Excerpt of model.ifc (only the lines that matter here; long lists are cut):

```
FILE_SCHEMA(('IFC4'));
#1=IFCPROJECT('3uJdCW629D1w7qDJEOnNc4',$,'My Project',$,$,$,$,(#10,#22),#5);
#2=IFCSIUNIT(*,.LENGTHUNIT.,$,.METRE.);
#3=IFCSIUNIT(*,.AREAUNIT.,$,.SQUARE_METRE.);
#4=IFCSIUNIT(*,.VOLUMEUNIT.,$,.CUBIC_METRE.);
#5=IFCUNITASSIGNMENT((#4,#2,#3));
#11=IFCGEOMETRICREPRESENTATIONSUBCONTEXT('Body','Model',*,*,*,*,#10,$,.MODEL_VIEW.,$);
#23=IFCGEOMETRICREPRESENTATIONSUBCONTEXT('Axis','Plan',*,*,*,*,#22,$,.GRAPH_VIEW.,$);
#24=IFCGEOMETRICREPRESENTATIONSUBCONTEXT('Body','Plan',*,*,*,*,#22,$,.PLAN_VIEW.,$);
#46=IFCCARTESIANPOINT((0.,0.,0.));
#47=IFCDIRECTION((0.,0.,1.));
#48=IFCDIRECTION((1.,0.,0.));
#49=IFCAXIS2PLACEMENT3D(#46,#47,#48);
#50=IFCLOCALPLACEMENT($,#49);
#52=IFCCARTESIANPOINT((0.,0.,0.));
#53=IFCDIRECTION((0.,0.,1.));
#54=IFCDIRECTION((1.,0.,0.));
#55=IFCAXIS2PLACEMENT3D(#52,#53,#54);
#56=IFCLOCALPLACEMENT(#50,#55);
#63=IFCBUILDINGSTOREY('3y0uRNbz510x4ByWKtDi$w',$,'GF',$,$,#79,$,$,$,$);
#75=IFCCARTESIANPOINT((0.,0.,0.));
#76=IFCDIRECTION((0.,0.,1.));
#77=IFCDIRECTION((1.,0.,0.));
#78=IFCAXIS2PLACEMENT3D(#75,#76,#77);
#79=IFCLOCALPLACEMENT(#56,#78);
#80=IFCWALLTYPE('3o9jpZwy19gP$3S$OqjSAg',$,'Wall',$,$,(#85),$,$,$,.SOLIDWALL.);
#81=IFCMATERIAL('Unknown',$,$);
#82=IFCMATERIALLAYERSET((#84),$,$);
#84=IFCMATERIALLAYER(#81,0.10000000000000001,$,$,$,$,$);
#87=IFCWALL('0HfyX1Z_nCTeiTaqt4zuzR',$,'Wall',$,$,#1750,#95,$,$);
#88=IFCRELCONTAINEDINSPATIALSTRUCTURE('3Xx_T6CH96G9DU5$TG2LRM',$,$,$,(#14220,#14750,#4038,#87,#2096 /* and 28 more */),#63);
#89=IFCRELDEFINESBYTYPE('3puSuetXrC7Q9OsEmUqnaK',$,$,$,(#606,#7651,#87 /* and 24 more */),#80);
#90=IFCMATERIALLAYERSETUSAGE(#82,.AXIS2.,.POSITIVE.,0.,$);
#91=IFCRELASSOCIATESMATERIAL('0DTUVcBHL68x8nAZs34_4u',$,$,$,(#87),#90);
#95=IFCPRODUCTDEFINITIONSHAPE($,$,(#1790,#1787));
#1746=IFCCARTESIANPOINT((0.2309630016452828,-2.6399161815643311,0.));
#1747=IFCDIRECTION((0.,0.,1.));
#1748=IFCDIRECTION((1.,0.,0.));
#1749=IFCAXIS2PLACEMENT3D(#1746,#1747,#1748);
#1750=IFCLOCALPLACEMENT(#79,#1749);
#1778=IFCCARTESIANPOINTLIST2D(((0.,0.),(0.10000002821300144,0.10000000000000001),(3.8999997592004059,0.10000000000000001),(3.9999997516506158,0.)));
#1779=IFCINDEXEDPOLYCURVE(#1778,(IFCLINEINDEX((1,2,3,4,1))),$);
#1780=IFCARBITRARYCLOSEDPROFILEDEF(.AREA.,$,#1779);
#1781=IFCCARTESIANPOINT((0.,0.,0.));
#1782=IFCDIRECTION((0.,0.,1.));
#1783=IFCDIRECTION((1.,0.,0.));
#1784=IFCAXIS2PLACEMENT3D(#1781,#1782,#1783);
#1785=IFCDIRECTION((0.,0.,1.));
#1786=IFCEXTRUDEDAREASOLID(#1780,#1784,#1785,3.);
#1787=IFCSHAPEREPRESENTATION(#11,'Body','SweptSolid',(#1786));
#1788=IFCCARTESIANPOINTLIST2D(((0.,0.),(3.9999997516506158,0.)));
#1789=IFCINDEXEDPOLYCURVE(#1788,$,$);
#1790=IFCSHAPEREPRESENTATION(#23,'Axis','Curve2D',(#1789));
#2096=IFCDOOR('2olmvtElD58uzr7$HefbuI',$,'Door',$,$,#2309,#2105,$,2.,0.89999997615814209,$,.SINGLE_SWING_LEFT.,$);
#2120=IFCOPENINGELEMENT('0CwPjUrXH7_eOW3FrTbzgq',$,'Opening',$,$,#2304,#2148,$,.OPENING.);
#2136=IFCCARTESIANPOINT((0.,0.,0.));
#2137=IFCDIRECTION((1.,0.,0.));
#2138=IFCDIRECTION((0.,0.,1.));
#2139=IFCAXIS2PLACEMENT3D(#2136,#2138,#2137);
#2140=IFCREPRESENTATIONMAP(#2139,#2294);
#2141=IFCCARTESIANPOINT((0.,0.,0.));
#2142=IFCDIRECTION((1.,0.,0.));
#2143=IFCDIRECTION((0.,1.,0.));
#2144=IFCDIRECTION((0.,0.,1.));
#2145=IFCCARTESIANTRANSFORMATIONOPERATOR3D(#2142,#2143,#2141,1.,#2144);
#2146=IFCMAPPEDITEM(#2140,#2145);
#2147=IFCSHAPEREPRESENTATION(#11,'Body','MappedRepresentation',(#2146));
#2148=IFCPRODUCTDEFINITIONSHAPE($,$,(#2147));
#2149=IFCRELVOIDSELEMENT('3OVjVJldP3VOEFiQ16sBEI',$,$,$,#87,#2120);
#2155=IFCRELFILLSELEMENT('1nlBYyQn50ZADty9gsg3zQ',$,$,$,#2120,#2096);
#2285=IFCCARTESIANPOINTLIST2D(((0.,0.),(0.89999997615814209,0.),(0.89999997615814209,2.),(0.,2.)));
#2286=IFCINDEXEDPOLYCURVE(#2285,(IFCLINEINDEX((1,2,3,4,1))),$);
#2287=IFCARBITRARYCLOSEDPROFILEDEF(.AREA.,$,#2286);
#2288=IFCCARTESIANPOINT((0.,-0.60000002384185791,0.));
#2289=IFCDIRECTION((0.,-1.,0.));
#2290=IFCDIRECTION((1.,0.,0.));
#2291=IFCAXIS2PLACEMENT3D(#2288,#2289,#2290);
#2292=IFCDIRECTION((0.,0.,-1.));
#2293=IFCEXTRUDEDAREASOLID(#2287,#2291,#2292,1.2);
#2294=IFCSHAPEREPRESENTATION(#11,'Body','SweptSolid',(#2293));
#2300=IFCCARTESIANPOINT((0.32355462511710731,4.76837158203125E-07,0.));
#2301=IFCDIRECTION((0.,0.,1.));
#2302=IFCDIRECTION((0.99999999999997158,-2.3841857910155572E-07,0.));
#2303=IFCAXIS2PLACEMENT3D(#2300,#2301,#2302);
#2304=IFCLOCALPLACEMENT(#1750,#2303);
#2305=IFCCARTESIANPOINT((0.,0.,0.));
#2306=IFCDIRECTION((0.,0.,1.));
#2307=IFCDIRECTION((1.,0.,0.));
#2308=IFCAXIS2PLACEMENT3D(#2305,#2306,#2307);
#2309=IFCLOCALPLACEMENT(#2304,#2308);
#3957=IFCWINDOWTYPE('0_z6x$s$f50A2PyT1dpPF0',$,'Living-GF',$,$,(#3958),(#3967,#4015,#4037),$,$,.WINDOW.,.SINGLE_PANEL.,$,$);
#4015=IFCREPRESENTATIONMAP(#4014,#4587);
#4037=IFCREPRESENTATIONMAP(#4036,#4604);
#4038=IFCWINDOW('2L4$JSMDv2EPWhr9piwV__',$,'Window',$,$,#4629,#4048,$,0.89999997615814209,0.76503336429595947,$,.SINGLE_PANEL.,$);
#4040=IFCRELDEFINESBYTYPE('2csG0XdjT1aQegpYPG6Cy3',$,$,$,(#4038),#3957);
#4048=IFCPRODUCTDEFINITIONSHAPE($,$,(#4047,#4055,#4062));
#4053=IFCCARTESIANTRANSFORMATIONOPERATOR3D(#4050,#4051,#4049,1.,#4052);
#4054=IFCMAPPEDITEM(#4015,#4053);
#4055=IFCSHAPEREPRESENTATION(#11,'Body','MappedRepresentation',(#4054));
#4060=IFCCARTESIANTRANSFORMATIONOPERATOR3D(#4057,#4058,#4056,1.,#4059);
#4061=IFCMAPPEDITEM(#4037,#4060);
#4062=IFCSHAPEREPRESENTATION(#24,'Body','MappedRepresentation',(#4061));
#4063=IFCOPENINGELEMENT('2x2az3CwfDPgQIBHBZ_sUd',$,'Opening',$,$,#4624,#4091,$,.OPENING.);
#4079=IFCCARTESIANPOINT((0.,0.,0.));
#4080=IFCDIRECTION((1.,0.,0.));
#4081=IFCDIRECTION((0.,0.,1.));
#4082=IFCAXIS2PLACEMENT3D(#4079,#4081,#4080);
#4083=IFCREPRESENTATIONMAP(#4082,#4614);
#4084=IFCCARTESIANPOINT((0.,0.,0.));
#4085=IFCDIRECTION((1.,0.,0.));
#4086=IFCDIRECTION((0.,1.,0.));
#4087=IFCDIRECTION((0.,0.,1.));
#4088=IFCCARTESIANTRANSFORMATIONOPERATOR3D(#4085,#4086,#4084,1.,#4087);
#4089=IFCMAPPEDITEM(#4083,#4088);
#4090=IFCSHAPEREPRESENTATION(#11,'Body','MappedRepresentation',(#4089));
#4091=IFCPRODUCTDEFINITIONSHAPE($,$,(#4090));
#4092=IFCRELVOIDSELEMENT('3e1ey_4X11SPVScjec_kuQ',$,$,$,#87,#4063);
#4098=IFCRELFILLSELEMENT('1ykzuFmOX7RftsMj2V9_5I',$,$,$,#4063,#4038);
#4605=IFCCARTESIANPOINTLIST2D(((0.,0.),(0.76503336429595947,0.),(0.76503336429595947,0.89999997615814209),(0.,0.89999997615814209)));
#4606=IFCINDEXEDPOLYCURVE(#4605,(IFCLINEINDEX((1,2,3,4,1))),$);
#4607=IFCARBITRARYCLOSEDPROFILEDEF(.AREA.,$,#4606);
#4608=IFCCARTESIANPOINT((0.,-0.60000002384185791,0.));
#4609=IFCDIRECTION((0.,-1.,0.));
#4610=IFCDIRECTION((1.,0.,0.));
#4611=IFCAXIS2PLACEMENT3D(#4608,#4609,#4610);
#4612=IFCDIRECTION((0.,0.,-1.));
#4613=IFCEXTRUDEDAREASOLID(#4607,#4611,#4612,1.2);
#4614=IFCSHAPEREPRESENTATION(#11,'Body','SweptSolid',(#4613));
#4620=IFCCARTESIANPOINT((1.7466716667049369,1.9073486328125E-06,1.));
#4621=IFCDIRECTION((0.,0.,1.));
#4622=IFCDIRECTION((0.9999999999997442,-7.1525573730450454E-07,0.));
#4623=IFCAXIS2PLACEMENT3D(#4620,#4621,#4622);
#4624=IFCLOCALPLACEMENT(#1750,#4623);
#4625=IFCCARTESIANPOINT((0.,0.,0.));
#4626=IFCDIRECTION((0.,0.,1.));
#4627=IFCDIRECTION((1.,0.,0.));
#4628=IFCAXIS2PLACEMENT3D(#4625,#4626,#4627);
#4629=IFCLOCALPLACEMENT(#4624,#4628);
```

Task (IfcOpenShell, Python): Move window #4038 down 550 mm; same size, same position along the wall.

```python
import numpy as np
import ifcopenshell
import ifcopenshell.api.geometry
import ifcopenshell.util.placement
import ifcopenshell.util.unit

model = ifcopenshell.open("model.ifc")
unit_scale = ifcopenshell.util.unit.calculate_unit_scale(model)

window = model.by_guid("2L4$JSMDv2EPWhr9piwV__")
opening = window.FillsVoids[0].RelatingOpeningElement
dz = -0.55 / unit_scale

shift = np.array([0.0, 0.0, dz])
# The window is placed relative to its opening, so it follows when the opening moves.
matrix = ifcopenshell.util.placement.get_local_placement(opening.ObjectPlacement)
matrix[:3, 3] += shift
ifcopenshell.api.geometry.edit_object_placement(
    model, product=opening, matrix=matrix, is_si=False, should_transform_children=True
)

print(f"moved by {dz * unit_scale:+.3f} m")

model.write("model_updated.ifc")
```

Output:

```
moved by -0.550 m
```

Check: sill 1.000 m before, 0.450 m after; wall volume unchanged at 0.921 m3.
